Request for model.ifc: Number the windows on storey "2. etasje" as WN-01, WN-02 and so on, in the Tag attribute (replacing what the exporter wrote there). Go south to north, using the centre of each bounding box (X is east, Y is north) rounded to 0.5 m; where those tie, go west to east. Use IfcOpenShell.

First a look at what the model holds.

```python
import ifcopenshell
import ifcopenshell.util.element
import ifcopenshell.util.placement

model = ifcopenshell.open("model.ifc")
print(model.schema)
storey = next(s for s in model.by_type("IfcBuildingStorey") if s.Name == "2. etasje")
windows = [e for e in ifcopenshell.util.element.get_decomposition(storey) if e.is_a("IfcWindow")]
for e in sorted(windows, key=lambda e: e.id()):
    origin = ifcopenshell.util.placement.get_local_placement(e.ObjectPlacement)[:3, 3]
    print(e.id(), e.Tag, e.Name, origin.round(2) + 0.0, sep=" | ")
```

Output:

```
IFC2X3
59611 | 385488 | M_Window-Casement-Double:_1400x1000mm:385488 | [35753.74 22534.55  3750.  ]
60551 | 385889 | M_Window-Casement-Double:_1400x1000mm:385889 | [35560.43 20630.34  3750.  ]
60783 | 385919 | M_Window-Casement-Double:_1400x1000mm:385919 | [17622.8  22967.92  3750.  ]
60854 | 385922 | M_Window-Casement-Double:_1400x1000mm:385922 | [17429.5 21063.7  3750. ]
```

```python
import ifcopenshell
import ifcopenshell.geom
import ifcopenshell.util.element
import ifcopenshell.util.shape

model = ifcopenshell.open("model.ifc")
settings = ifcopenshell.geom.settings()
settings.set("use-world-coords", True)


def centre(element):
    shape = ifcopenshell.geom.create_shape(settings, element)
    return ifcopenshell.util.shape.get_bbox_centroid(shape.geometry)


storey = next(s for s in model.by_type("IfcBuildingStorey") if s.Name == "2. etasje")
windows = [e for e in ifcopenshell.util.element.get_decomposition(storey) if e.is_a("IfcWindow")]

# Insertion points can sit at a corner or the storey origin, so sort by the geometry (in metres).
centres = {e: centre(e) for e in windows}
windows.sort(key=lambda e: (round(centres[e][1] / 0.5), centres[e][0]))

for i, e in enumerate(windows, start=1):
    number = f"WN-{i:02d}"
    e.Tag = number
    print(e.id(), number)

model.write("model_edited.ifc")
```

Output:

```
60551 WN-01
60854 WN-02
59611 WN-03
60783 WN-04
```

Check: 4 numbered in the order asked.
